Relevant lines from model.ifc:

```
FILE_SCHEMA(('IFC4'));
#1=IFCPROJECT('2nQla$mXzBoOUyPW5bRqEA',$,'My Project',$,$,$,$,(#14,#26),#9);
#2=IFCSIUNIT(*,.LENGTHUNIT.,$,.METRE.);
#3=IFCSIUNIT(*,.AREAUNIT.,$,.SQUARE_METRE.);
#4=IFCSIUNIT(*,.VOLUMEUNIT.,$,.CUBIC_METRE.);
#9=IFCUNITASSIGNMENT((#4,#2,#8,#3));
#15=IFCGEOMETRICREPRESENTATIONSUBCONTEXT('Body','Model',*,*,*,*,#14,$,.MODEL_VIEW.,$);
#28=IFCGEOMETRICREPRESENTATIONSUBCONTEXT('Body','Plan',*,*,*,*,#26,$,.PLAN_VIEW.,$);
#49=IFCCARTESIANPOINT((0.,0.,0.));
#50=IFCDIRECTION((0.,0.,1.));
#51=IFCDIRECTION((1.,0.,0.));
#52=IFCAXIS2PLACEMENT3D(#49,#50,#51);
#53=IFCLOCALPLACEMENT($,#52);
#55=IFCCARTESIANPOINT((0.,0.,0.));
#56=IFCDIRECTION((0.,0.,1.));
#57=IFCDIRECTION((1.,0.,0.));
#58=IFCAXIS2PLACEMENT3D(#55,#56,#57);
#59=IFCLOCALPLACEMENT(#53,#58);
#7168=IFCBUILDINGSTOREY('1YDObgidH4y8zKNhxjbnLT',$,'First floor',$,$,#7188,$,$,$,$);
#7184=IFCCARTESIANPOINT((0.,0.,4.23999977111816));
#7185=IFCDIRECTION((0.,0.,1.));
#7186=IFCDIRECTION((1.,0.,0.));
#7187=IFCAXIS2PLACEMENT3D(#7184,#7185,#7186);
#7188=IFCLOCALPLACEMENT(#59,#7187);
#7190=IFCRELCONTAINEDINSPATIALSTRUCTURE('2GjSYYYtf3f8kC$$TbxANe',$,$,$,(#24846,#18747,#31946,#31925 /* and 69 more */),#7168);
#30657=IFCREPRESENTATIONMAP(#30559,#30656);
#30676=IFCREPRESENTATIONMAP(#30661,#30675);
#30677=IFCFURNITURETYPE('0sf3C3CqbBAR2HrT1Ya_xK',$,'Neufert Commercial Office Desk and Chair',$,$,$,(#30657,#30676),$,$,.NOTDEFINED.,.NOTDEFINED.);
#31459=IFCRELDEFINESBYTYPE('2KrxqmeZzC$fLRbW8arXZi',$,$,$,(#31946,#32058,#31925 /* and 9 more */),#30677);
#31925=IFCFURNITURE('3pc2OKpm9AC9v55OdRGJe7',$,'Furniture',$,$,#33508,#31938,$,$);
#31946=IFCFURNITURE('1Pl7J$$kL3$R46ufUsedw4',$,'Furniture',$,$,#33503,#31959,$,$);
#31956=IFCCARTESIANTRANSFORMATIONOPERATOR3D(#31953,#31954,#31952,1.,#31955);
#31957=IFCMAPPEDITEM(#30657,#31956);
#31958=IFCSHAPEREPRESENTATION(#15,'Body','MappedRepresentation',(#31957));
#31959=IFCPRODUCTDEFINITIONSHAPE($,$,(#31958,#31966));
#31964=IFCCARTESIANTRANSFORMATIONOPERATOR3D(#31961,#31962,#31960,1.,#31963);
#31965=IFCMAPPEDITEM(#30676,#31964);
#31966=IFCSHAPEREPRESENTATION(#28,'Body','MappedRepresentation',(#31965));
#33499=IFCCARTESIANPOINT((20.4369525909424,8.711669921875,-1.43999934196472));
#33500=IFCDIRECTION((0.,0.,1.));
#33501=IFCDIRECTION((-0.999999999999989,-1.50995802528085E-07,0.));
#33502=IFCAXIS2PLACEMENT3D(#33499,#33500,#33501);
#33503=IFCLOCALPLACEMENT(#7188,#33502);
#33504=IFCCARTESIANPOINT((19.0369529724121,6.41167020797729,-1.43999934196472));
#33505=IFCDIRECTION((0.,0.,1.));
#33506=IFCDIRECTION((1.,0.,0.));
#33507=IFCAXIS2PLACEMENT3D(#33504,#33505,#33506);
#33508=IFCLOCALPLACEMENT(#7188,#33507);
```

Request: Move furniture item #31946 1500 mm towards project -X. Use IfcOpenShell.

```python
import ifcopenshell
import ifcopenshell.api.geometry
import ifcopenshell.util.placement

model = ifcopenshell.open("model.ifc")

item = model.by_guid("1Pl7J$$kL3$R46ufUsedw4")
matrix = ifcopenshell.util.placement.get_local_placement(item.ObjectPlacement)
matrix[0, 3] -= 1.5
ifcopenshell.api.geometry.edit_object_placement(model, product=item, matrix=matrix, is_si=False)

print(ifcopenshell.util.placement.get_local_placement(item.ObjectPlacement).round(3) + 0.0)

model.write("model-out.ifc")
```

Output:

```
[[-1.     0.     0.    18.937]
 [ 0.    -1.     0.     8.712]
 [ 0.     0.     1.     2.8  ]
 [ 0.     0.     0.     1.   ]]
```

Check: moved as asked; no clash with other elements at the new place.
